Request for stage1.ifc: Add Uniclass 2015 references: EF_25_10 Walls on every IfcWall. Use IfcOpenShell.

First a look at what the model holds.

```python
import ifcopenshell

model = ifcopenshell.open("stage1.ifc")
print(model.schema)
print("classifications:", [c.Name for c in model.by_type("IfcClassification")])
for ifc_class in ("IfcDoor", "IfcRoof", "IfcStair", "IfcWall", "IfcWindow"):
    print(ifc_class, len(model.by_type(ifc_class)))
```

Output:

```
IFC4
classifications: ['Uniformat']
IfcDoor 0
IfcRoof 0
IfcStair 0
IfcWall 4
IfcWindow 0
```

```python
import ifcopenshell
import ifcopenshell.api.classification

model = ifcopenshell.open("stage1.ifc")

system = ifcopenshell.api.classification.add_classification(model, classification="Uniclass 2015")

codes = {
    "IfcWall": ("EF_25_10", "Walls"),
}
for ifc_class, (code, name) in codes.items():
    products = model.by_type(ifc_class)
    ifcopenshell.api.classification.add_reference(
        model, products=products, classification=system, identification=code, name=name
    )
    print(code, len(products))

model.write("stage1_updated.ifc")
```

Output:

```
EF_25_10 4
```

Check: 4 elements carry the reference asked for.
